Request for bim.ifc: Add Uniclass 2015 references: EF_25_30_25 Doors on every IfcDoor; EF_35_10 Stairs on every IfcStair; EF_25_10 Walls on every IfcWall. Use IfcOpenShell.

First a look at what the model holds.

```python
import ifcopenshell

model = ifcopenshell.open("bim.ifc")
print(model.schema)
print("classifications:", [c.Name for c in model.by_type("IfcClassification")])
for ifc_class in ("IfcDoor", "IfcRoof", "IfcStair", "IfcWall", "IfcWindow"):
    print(ifc_class, len(model.by_type(ifc_class)))
```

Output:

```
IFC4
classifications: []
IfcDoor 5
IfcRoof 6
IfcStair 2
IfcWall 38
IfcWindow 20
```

```python
import ifcopenshell
import ifcopenshell.api.classification

model = ifcopenshell.open("bim.ifc")

system = ifcopenshell.api.classification.add_classification(model, classification="Uniclass 2015")

codes = {
    "IfcDoor": ("EF_25_30_25", "Doors"),
    "IfcStair": ("EF_35_10", "Stairs"),
    "IfcWall": ("EF_25_10", "Walls"),
}
for ifc_class, (code, name) in codes.items():
    products = model.by_type(ifc_class)
    ifcopenshell.api.classification.add_reference(
        model, products=products, classification=system, identification=code, name=name
    )
    print(code, len(products))

model.write("bim_updated.ifc")
```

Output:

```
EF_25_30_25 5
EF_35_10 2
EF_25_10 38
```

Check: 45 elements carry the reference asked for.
